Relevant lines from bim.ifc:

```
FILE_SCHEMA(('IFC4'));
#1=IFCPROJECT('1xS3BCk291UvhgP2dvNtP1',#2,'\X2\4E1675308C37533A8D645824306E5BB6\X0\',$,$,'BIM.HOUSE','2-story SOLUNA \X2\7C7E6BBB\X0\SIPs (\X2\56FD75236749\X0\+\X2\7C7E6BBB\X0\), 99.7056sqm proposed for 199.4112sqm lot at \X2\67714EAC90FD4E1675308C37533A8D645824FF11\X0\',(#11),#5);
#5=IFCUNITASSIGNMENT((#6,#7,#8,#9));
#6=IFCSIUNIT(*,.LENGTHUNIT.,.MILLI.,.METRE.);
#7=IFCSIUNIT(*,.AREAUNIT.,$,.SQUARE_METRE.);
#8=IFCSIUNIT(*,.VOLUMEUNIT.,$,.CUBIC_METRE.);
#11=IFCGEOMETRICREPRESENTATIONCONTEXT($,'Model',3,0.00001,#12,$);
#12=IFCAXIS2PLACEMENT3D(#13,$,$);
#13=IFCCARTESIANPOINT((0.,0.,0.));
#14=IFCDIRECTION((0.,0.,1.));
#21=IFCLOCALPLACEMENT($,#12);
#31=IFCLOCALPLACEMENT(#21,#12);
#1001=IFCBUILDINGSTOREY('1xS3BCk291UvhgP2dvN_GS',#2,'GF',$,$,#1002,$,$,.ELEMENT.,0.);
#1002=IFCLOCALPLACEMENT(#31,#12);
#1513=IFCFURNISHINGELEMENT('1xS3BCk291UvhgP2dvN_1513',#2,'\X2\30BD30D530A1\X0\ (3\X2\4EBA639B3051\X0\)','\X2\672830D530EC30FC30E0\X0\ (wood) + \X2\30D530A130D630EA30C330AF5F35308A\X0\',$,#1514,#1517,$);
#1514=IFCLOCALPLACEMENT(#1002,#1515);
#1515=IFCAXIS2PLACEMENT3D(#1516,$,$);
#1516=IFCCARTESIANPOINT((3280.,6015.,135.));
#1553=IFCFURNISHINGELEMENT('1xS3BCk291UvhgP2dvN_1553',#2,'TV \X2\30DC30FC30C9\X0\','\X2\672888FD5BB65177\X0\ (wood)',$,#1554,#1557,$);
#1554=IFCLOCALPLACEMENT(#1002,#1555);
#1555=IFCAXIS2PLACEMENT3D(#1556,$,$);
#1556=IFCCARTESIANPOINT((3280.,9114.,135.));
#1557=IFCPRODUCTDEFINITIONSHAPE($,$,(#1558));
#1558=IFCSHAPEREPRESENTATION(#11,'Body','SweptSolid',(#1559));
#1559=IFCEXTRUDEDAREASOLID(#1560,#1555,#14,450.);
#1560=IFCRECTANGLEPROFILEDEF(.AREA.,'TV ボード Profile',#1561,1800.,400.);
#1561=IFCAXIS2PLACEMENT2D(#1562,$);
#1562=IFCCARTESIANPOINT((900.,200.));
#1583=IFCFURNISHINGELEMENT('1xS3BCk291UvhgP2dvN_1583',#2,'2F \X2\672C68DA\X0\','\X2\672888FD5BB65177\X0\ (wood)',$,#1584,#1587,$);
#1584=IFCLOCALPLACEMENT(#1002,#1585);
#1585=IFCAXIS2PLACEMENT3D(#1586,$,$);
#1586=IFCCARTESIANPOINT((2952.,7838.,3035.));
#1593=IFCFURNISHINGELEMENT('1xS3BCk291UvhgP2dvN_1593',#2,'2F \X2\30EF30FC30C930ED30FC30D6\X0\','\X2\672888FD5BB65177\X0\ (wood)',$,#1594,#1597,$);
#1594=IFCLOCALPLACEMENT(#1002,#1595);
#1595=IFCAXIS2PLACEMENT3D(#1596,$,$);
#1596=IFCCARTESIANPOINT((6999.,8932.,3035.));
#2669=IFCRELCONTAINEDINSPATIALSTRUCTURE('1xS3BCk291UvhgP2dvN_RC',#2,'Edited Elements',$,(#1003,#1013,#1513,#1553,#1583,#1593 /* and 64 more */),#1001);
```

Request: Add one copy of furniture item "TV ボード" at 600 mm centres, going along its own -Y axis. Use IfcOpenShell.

```python
import ifcopenshell
import ifcopenshell.api.geometry
import ifcopenshell.api.root
import ifcopenshell.util.element
import ifcopenshell.util.placement

model = ifcopenshell.open("bim.ifc")


def reuse_history(source, copy):
    """copy_class also copies each property set's owner history, people and application; keep the originals."""
    for rel in copy.IsDefinedBy:
        if rel.is_a("IfcRelDefinesByProperties") and (history := rel.RelatingPropertyDefinition.OwnerHistory):
            rel.RelatingPropertyDefinition.OwnerHistory = source.OwnerHistory
            ifcopenshell.util.element.remove_deep2(model, history)


source = model.by_id(1553)
base = ifcopenshell.util.placement.get_local_placement(source.ObjectPlacement)
step = -base[:3, 1] * 600.0

for i in range(1, 2):
    copy = ifcopenshell.api.root.copy_class(model, product=source)
    copy.Representation = ifcopenshell.util.element.copy_deep(
        model, source.Representation, exclude=["IfcGeometricRepresentationContext", "IfcRepresentationMap"]
    )
    reuse_history(source, copy)
    matrix = base.copy()
    matrix[:3, 3] += i * step
    print("added at", matrix[:3, 3].round(3) + 0.0)
    ifcopenshell.api.geometry.edit_object_placement(model, product=copy, matrix=matrix, is_si=False)

model.write("bim-out.ifc")
```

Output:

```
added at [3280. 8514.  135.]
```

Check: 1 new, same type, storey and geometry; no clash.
